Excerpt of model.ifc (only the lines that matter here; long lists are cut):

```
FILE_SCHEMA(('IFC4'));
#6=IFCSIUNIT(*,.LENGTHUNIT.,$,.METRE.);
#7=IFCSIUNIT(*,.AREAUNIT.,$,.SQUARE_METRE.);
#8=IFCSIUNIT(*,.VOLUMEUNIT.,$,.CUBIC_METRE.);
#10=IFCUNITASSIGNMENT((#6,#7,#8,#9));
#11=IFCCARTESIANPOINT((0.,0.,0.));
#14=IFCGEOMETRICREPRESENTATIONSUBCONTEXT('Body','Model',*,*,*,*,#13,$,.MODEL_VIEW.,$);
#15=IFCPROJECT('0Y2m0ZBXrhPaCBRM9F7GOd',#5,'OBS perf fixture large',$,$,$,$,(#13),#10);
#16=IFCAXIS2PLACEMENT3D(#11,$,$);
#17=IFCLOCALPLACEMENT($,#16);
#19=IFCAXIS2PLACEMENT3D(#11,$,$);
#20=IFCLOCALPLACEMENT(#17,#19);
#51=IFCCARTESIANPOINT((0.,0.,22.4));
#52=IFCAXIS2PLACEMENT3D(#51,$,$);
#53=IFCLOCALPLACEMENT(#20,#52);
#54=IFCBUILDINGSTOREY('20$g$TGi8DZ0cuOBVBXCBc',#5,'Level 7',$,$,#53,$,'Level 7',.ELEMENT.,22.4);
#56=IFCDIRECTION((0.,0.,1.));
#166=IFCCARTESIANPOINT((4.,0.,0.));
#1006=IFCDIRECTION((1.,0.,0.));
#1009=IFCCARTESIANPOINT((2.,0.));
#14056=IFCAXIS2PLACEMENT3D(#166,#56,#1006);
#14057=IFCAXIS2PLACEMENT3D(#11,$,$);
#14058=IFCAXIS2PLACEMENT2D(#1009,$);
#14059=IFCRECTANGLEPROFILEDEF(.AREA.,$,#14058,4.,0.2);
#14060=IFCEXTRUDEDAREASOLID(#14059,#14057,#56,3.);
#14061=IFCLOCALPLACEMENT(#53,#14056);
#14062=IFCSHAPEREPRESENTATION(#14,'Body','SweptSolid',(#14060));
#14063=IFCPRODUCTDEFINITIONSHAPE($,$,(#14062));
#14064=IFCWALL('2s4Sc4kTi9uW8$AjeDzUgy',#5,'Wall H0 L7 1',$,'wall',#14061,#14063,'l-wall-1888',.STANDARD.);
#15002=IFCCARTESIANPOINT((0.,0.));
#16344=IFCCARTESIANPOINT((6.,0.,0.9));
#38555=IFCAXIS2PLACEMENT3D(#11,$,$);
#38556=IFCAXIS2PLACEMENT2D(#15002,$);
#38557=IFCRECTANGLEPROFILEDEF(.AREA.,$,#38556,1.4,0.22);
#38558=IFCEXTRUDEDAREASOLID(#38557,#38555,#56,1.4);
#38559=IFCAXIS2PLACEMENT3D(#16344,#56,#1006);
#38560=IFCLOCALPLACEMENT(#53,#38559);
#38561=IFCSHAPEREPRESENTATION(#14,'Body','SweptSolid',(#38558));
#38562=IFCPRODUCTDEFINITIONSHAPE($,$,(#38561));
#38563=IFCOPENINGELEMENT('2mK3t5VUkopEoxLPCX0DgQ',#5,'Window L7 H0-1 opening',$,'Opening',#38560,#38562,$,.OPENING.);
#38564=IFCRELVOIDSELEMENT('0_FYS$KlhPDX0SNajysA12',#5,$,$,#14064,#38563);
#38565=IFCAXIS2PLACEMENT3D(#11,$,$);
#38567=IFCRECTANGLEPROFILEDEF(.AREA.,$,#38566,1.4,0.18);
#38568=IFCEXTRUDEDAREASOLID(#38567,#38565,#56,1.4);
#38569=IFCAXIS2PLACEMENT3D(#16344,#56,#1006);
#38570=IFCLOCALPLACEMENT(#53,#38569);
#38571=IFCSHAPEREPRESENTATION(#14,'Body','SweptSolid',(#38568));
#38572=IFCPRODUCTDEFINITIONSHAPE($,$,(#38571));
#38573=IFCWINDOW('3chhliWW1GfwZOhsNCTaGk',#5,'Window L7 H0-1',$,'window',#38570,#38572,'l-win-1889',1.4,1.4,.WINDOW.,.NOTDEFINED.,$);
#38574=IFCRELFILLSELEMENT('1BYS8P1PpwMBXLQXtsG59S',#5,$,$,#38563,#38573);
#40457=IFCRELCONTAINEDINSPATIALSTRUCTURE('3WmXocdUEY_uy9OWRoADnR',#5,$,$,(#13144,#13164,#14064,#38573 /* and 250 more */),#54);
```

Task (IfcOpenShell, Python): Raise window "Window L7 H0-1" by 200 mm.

```python
import numpy as np
import ifcopenshell
import ifcopenshell.api.geometry
import ifcopenshell.util.placement
import ifcopenshell.util.unit

model = ifcopenshell.open("model.ifc")
unit_scale = ifcopenshell.util.unit.calculate_unit_scale(model)

window = model.by_guid("3chhliWW1GfwZOhsNCTaGk")
opening = window.FillsVoids[0].RelatingOpeningElement
dz = 0.2 / unit_scale

shift = np.array([0.0, 0.0, dz])
# The window is not placed relative to its opening, so move both.
for product in (opening, window):
    matrix = ifcopenshell.util.placement.get_local_placement(product.ObjectPlacement)
    matrix[:3, 3] += shift
    ifcopenshell.api.geometry.edit_object_placement(model, product=product, matrix=matrix, is_si=False)

print(f"moved by {dz * unit_scale:+.3f} m")

model.write("model-out.ifc")
```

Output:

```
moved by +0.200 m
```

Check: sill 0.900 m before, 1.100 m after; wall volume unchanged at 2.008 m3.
